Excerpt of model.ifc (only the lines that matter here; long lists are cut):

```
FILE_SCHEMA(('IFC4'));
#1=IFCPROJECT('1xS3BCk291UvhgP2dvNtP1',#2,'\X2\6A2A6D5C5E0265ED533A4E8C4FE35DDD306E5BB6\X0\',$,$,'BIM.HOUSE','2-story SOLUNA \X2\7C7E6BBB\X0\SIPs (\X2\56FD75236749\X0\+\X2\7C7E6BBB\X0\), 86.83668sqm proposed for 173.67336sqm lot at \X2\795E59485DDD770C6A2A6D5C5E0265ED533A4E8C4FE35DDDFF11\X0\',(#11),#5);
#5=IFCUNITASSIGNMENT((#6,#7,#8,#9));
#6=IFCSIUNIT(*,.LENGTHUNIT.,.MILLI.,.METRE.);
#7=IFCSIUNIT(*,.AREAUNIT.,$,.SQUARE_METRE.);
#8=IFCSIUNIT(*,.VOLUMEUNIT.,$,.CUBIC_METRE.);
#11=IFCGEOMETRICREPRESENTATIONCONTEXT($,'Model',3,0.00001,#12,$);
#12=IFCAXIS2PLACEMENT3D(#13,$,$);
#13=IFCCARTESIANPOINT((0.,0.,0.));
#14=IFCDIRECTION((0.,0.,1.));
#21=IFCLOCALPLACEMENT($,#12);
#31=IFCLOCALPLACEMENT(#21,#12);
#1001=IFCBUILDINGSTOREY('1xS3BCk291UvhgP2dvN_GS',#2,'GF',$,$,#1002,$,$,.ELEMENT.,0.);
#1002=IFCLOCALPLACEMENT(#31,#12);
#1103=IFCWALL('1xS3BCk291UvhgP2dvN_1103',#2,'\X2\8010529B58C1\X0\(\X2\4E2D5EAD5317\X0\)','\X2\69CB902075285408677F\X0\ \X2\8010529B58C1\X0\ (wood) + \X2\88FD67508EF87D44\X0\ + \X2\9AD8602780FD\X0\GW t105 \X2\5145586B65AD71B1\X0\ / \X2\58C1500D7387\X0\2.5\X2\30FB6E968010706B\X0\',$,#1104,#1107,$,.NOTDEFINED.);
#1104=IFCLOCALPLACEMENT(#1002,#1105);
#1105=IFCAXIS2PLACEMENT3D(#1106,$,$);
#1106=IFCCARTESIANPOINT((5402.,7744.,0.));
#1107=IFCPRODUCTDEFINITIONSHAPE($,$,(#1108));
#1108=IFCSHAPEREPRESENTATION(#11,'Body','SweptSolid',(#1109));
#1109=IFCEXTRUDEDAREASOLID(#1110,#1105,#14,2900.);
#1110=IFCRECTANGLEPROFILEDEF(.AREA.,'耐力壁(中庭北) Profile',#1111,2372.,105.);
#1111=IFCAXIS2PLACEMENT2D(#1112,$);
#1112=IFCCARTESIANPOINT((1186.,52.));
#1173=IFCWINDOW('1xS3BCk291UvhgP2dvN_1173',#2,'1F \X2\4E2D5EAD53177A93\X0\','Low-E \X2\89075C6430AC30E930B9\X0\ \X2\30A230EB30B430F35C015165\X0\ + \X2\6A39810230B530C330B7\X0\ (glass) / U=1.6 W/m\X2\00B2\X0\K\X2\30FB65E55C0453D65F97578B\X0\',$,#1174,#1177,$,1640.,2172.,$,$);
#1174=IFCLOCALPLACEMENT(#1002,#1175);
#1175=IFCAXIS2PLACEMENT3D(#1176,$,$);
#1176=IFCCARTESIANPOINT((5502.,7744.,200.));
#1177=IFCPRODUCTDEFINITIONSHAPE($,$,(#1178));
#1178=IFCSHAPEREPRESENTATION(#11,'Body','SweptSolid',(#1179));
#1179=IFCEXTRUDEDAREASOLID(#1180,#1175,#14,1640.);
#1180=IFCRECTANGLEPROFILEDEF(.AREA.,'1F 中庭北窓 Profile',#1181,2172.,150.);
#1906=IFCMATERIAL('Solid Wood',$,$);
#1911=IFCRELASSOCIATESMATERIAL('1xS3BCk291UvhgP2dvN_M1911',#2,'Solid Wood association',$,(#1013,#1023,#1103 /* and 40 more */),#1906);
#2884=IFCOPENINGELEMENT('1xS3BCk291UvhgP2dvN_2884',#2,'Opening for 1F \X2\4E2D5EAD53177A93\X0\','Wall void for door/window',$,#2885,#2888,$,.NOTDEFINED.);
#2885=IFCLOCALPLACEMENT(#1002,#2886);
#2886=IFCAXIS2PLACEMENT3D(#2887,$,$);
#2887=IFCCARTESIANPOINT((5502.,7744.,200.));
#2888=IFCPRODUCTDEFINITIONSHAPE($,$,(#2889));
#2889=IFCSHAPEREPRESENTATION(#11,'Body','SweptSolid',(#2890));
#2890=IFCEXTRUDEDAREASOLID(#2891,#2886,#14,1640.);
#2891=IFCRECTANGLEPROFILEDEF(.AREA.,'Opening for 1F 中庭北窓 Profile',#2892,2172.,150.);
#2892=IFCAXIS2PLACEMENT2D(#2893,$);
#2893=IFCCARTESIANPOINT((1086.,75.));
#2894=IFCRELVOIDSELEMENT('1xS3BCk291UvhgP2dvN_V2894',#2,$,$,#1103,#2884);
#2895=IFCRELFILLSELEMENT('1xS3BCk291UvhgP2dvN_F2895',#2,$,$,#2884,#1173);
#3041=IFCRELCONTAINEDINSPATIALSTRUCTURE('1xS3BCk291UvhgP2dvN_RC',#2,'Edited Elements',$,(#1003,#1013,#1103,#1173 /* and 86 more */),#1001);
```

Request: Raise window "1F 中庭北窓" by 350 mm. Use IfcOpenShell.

```python
import numpy as np
import ifcopenshell
import ifcopenshell.api.geometry
import ifcopenshell.util.placement
import ifcopenshell.util.unit

model = ifcopenshell.open("model.ifc")
unit_scale = ifcopenshell.util.unit.calculate_unit_scale(model)

window = model.by_guid("1xS3BCk291UvhgP2dvN_1173")
opening = window.FillsVoids[0].RelatingOpeningElement
dz = 0.35 / unit_scale

shift = np.array([0.0, 0.0, dz])
# The window is not placed relative to its opening, so move both.
for product in (opening, window):
    matrix = ifcopenshell.util.placement.get_local_placement(product.ObjectPlacement)
    matrix[:3, 3] += shift
    ifcopenshell.api.geometry.edit_object_placement(model, product=product, matrix=matrix, is_si=False)

print(f"moved by {dz * unit_scale:+.3f} m")

model.write("model_v2.ifc")
```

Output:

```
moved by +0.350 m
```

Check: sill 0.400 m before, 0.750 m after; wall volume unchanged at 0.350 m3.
